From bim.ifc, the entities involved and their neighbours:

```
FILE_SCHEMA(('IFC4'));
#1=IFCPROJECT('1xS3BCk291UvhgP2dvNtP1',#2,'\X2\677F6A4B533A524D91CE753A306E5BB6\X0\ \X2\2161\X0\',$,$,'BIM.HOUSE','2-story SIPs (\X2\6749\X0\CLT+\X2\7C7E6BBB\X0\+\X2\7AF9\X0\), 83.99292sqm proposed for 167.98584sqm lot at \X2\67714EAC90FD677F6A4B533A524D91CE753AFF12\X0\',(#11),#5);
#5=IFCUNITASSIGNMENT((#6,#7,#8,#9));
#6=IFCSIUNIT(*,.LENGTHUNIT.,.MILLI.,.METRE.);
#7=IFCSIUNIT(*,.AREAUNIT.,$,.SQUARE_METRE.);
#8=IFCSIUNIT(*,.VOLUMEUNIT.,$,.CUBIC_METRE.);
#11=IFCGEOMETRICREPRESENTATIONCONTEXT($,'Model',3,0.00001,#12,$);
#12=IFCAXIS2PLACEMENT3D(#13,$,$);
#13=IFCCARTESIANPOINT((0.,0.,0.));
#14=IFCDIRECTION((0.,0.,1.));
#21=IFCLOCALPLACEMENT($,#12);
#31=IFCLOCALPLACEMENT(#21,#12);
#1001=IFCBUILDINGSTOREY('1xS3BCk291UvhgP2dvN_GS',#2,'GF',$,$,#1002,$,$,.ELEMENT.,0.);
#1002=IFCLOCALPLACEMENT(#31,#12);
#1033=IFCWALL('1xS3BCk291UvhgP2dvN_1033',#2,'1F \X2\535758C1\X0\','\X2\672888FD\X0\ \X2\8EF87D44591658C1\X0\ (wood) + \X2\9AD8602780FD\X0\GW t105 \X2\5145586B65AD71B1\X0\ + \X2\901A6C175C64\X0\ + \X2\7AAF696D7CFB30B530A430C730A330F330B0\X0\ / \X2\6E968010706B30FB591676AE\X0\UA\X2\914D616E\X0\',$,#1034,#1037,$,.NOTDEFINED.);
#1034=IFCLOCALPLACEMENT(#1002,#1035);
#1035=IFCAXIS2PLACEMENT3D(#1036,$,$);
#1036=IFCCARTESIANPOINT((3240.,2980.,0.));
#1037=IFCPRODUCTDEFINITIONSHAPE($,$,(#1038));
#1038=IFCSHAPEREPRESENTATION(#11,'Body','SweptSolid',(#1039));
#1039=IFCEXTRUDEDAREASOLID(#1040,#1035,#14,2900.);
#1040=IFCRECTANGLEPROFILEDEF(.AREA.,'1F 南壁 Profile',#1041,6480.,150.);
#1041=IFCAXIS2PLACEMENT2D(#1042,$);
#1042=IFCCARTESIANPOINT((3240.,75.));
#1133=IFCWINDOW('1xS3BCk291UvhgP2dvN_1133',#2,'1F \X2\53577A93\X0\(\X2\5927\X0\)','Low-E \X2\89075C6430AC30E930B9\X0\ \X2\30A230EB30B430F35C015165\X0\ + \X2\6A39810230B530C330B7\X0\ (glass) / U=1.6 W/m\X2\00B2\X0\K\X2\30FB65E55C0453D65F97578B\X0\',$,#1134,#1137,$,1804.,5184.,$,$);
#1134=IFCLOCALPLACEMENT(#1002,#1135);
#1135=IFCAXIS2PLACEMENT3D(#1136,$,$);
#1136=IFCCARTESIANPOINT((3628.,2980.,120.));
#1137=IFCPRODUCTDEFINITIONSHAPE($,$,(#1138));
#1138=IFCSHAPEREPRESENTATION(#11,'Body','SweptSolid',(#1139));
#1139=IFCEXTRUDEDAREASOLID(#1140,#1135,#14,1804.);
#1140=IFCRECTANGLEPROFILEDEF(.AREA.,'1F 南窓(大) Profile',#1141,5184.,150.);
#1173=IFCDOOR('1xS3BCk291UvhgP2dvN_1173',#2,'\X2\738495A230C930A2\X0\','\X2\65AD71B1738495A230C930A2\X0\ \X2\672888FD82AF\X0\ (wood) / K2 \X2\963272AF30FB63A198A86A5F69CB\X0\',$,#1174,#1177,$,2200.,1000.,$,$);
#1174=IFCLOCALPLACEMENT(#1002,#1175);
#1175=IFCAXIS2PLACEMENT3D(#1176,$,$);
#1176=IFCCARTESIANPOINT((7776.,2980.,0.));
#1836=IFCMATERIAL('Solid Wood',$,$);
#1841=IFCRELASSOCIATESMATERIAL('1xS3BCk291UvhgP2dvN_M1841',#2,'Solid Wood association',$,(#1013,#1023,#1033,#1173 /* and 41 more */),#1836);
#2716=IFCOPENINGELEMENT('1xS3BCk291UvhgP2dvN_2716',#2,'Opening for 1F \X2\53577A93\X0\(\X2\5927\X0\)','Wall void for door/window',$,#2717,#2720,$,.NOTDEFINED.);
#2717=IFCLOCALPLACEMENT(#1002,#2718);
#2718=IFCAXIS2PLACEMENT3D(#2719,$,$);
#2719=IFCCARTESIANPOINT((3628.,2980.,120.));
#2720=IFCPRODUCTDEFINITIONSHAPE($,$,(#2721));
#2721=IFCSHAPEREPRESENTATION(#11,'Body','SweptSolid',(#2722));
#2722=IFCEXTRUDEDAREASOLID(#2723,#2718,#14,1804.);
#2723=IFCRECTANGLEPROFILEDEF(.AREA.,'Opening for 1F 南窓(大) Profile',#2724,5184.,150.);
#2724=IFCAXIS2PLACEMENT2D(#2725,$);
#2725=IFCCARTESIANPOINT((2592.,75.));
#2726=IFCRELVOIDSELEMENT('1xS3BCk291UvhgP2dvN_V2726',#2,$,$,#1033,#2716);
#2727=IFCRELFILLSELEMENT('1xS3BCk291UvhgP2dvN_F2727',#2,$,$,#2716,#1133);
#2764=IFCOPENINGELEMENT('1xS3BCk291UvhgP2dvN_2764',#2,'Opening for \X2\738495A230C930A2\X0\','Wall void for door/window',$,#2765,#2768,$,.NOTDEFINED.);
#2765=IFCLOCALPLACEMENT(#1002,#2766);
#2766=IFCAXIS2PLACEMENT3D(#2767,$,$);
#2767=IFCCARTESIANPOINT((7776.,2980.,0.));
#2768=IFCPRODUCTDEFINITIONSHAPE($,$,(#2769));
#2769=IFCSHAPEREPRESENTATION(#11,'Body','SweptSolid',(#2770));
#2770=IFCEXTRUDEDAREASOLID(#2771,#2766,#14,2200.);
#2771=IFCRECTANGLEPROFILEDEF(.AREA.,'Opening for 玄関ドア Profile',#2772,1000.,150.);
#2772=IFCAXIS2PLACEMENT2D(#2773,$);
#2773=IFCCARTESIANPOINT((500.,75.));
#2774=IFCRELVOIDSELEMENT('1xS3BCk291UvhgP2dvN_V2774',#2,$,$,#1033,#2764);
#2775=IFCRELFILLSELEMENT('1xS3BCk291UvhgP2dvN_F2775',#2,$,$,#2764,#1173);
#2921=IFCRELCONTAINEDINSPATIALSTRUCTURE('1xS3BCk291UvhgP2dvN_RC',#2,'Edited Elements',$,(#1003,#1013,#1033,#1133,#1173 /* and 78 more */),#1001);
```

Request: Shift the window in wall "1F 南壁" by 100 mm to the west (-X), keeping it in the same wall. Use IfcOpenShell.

```python
import ifcopenshell
import ifcopenshell.api.geometry
import ifcopenshell.util.placement
import ifcopenshell.util.unit

model = ifcopenshell.open("bim.ifc")
unit_scale = ifcopenshell.util.unit.calculate_unit_scale(model)

window = model.by_id(1133)
opening = window.FillsVoids[0].RelatingOpeningElement
wall = opening.VoidsElements[0].RelatingBuildingElement

wall_matrix = ifcopenshell.util.placement.get_local_placement(wall.ObjectPlacement)
shift = wall_matrix[:3, 0] * -0.1 / unit_scale
before = ifcopenshell.util.placement.get_local_placement(window.ObjectPlacement)[:3, 3].copy()

# The window is not placed relative to its opening, so move both.
for product in (opening, window):
    matrix = ifcopenshell.util.placement.get_local_placement(product.ObjectPlacement)
    matrix[:3, 3] += shift
    ifcopenshell.api.geometry.edit_object_placement(model, product=product, matrix=matrix, is_si=False)

after = ifcopenshell.util.placement.get_local_placement(window.ObjectPlacement)[:3, 3]
print("window moved by", (after - before).round(3) + 0.0)

model.write("bim_edited.ifc")
```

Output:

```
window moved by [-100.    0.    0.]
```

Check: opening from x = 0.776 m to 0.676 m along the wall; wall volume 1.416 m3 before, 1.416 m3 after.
